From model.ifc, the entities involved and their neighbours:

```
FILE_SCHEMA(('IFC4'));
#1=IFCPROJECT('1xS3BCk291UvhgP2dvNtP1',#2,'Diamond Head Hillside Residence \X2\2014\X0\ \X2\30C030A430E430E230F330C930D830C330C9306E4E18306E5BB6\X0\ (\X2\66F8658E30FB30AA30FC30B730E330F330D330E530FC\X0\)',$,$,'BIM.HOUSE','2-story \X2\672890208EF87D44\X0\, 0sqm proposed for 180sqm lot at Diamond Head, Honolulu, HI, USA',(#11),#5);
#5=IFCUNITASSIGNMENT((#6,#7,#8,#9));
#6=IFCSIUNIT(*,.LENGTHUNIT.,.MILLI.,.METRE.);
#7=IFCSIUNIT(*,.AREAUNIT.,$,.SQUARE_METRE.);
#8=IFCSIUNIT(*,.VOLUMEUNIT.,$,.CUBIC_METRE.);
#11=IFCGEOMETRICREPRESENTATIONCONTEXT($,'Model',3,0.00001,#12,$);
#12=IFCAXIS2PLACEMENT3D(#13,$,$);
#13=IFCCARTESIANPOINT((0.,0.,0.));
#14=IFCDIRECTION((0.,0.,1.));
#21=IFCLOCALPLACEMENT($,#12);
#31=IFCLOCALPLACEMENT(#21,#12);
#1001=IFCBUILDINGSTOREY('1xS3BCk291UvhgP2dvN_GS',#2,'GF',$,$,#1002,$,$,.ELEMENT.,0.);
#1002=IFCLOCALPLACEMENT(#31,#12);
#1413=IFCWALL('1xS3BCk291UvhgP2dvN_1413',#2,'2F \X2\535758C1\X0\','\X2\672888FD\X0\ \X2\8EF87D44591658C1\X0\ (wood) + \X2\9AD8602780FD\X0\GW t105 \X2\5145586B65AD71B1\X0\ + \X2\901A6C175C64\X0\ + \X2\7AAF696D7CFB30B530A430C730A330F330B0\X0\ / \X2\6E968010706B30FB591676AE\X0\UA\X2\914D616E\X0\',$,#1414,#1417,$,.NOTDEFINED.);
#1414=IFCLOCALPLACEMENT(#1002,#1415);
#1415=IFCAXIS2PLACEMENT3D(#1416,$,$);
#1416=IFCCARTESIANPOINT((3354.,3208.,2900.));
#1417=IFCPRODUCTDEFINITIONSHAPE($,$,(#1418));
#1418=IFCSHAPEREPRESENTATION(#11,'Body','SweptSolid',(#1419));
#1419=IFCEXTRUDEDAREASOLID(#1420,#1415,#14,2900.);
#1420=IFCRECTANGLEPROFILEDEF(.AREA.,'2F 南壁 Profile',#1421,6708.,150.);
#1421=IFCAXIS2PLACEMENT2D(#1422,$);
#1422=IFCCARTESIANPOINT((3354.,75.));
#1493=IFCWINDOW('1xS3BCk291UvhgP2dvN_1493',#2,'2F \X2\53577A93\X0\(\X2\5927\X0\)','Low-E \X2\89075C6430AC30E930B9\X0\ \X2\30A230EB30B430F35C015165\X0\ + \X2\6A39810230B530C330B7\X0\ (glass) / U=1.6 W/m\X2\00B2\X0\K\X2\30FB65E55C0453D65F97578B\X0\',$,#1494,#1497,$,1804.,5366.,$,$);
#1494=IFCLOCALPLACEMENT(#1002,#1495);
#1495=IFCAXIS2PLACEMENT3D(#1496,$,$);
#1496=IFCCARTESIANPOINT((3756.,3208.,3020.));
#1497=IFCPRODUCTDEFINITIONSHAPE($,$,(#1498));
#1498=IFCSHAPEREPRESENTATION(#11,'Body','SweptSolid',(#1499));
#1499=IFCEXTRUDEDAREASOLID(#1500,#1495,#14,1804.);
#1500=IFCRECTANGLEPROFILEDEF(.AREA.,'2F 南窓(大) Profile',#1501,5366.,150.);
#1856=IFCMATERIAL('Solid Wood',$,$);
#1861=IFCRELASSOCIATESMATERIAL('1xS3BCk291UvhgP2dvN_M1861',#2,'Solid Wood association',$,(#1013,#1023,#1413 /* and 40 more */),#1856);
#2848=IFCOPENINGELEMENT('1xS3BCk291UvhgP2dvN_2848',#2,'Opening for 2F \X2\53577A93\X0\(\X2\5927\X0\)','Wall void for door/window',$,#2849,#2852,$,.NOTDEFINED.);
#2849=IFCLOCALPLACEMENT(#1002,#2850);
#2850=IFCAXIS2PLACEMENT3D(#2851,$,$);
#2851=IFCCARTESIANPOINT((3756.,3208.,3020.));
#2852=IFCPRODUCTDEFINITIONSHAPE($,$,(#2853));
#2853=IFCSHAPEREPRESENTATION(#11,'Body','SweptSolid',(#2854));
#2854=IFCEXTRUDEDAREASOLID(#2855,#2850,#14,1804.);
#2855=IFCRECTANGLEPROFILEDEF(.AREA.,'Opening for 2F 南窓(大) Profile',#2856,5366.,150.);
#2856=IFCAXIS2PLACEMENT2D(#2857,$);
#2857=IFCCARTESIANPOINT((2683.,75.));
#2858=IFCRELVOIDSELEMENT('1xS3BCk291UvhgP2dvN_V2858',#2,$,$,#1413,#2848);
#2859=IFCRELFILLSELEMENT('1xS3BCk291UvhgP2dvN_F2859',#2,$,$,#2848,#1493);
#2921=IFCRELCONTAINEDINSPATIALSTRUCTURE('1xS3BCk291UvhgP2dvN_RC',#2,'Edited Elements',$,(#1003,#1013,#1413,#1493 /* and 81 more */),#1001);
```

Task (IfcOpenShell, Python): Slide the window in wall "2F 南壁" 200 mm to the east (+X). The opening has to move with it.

```python
import ifcopenshell
import ifcopenshell.api.geometry
import ifcopenshell.util.placement

model = ifcopenshell.open("model.ifc")

window = model.by_guid("1xS3BCk291UvhgP2dvN_1493")
opening = window.FillsVoids[0].RelatingOpeningElement
wall = opening.VoidsElements[0].RelatingBuildingElement

wall_matrix = ifcopenshell.util.placement.get_local_placement(wall.ObjectPlacement)
shift = wall_matrix[:3, 0] * 200.0
before = ifcopenshell.util.placement.get_local_placement(window.ObjectPlacement)[:3, 3].copy()

# The window is not placed relative to its opening, so move both.
for product in (opening, window):
    matrix = ifcopenshell.util.placement.get_local_placement(product.ObjectPlacement)
    matrix[:3, 3] += shift
    ifcopenshell.api.geometry.edit_object_placement(model, product=product, matrix=matrix, is_si=False)

after = ifcopenshell.util.placement.get_local_placement(window.ObjectPlacement)[:3, 3]
print("window moved by", (after - before).round(3) + 0.0)

model.write("model_v2.ifc")
```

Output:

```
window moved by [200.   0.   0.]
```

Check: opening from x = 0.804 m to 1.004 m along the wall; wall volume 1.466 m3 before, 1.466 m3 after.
